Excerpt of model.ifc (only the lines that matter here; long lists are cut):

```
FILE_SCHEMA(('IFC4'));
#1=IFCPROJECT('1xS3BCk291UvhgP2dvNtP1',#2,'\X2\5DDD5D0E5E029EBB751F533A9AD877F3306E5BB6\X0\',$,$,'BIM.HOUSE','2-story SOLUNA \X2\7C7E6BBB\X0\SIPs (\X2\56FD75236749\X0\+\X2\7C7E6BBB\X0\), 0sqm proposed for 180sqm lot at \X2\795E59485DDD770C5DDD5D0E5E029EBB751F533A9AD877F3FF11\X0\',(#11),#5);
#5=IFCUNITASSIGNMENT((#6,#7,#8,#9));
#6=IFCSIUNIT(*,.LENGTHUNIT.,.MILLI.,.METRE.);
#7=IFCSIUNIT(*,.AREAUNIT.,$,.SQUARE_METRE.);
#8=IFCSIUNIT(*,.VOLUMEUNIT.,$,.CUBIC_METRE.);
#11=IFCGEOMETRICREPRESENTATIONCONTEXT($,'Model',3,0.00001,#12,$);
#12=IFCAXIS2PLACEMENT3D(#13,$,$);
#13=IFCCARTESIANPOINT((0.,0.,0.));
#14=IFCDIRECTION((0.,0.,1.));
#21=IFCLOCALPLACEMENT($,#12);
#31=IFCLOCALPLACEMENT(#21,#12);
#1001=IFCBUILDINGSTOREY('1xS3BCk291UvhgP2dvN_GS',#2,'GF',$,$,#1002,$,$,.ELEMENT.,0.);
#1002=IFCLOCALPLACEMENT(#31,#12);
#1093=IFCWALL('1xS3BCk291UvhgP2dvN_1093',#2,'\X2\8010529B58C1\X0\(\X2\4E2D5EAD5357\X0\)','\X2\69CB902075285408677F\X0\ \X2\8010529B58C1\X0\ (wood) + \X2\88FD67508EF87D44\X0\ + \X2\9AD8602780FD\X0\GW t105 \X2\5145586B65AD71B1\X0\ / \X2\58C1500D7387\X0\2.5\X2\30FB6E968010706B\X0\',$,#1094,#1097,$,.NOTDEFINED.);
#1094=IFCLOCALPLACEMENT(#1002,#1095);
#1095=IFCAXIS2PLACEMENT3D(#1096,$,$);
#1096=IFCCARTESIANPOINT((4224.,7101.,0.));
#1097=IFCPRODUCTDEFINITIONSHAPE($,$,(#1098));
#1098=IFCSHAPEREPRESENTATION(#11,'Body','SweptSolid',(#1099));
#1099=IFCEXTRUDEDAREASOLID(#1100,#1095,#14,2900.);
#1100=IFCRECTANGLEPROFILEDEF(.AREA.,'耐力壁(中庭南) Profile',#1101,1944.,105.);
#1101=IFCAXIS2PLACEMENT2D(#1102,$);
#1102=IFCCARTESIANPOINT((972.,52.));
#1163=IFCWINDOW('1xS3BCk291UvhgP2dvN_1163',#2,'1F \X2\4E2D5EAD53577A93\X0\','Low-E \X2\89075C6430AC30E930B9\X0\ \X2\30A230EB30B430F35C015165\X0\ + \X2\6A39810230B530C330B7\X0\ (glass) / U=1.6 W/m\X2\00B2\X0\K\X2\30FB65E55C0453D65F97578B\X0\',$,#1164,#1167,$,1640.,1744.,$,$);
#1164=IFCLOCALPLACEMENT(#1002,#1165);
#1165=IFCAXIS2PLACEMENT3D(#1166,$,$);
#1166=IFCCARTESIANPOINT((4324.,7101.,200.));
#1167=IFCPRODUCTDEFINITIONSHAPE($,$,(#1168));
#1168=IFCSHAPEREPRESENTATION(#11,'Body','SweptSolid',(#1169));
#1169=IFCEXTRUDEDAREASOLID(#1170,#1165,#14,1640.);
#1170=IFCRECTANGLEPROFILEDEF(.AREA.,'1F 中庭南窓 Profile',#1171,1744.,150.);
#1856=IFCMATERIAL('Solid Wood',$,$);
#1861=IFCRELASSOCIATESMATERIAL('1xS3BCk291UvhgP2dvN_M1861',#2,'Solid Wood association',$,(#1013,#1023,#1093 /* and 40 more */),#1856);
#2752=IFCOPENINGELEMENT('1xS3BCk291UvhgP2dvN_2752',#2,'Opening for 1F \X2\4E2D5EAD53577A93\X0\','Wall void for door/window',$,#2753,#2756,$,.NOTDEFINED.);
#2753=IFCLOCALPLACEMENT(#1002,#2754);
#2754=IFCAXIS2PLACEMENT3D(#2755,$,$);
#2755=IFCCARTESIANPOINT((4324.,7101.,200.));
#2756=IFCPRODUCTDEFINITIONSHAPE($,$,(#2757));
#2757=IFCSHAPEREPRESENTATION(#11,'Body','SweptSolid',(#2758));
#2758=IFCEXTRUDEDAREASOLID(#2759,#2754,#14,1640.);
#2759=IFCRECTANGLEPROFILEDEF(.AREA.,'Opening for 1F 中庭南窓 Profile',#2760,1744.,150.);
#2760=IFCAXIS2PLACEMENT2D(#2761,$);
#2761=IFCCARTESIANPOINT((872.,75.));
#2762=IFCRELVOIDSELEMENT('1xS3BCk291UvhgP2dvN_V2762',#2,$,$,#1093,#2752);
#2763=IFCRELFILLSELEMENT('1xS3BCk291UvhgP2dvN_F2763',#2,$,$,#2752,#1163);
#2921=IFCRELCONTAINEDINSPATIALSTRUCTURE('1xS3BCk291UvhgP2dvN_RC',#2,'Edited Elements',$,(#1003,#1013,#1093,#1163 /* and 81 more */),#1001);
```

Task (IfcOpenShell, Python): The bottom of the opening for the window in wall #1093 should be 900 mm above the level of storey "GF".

```python
import numpy as np
import ifcopenshell
import ifcopenshell.api.geometry
import ifcopenshell.geom
import ifcopenshell.util.element
import ifcopenshell.util.placement
import ifcopenshell.util.shape
import ifcopenshell.util.unit

model = ifcopenshell.open("model.ifc")
unit_scale = ifcopenshell.util.unit.calculate_unit_scale(model)

window = model.by_guid("1xS3BCk291UvhgP2dvN_1163")
opening = window.FillsVoids[0].RelatingOpeningElement
storey = ifcopenshell.util.element.get_container(window, ifc_class="IfcBuildingStorey")
level = ifcopenshell.util.placement.get_local_placement(storey.ObjectPlacement)[2, 3]

# The opening's origin need not be at the sill, so measure its lowest point.
shape = ifcopenshell.geom.create_shape(ifcopenshell.geom.settings(), opening)
bottom = ifcopenshell.util.shape.get_shape_bottom_elevation(shape, shape.geometry) / unit_scale
dz = level + 0.9 / unit_scale - bottom

shift = np.array([0.0, 0.0, dz])
# The window is not placed relative to its opening, so move both.
for product in (opening, window):
    matrix = ifcopenshell.util.placement.get_local_placement(product.ObjectPlacement)
    matrix[:3, 3] += shift
    ifcopenshell.api.geometry.edit_object_placement(model, product=product, matrix=matrix, is_si=False)

print(f"moved by {dz * unit_scale:+.3f} m")

model.write("model_edited.ifc")
```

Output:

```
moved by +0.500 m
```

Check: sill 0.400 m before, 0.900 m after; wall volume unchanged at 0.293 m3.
